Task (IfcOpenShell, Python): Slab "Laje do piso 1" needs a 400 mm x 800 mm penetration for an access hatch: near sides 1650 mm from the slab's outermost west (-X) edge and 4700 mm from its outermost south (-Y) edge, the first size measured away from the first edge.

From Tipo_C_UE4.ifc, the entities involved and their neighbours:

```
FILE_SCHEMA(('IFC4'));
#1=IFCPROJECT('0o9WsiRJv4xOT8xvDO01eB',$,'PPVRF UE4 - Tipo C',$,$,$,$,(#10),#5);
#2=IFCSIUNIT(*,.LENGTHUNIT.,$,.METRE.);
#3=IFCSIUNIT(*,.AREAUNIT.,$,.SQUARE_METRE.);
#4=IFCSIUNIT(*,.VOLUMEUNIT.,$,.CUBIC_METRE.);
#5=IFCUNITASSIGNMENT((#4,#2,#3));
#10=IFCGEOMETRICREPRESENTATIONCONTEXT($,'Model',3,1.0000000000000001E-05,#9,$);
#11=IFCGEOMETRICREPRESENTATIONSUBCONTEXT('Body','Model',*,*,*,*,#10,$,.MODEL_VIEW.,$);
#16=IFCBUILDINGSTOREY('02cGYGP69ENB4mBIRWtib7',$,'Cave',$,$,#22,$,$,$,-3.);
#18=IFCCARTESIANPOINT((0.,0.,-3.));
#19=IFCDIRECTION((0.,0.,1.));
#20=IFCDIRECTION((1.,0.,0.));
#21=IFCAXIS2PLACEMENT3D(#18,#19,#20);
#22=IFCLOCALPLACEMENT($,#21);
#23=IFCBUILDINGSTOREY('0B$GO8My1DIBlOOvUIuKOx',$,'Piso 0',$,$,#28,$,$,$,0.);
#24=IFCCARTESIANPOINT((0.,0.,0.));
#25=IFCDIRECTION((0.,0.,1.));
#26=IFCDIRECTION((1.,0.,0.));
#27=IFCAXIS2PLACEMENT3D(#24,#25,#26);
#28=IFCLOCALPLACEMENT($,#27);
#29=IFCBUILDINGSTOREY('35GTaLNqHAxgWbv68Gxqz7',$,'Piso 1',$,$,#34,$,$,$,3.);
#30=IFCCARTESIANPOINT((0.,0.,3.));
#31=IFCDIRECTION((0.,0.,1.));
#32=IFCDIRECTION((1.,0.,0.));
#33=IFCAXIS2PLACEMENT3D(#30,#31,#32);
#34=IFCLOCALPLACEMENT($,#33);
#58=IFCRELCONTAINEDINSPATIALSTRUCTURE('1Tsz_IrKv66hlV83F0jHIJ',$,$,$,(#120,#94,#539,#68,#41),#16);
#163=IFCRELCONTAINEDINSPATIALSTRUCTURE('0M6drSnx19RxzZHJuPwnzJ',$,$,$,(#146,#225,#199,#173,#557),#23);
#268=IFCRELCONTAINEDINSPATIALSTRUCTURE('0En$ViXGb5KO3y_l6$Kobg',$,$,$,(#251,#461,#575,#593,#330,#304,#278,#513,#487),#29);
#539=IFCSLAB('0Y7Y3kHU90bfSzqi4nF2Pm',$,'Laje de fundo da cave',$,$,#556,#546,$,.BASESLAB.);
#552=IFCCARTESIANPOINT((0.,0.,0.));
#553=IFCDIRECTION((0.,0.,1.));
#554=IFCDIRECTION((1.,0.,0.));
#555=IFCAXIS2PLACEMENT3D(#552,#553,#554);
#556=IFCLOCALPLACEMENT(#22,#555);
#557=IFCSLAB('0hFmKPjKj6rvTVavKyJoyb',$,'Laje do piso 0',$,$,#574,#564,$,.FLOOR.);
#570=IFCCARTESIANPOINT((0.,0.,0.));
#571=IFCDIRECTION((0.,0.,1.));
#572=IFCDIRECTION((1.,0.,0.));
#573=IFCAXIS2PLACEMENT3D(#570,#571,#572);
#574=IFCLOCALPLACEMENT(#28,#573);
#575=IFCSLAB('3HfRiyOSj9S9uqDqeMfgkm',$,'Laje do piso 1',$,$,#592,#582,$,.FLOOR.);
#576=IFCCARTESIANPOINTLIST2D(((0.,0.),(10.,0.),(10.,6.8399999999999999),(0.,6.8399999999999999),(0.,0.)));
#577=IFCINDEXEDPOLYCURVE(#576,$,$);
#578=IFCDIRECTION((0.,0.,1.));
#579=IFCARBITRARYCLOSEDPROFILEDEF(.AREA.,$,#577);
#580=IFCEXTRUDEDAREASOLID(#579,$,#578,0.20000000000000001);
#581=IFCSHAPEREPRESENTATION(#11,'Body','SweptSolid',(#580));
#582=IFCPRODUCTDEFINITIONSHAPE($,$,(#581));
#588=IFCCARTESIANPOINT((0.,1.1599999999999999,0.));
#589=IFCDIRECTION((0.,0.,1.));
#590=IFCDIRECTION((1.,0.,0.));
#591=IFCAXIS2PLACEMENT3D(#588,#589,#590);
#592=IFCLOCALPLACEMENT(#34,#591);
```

```python
import numpy as np
import ifcopenshell
import ifcopenshell.api.feature
import ifcopenshell.api.geometry
import ifcopenshell.api.root
import ifcopenshell.geom
import ifcopenshell.util.placement
import ifcopenshell.util.representation
import ifcopenshell.util.shape
import ifcopenshell.util.unit

model = ifcopenshell.open("Tipo_C_UE4.ifc")
unit_scale = ifcopenshell.util.unit.calculate_unit_scale(model)
settings = ifcopenshell.geom.settings()


def volume(element):
    """Net volume in cubic metres, openings subtracted."""
    shape = ifcopenshell.geom.create_shape(settings, element)
    return ifcopenshell.util.shape.get_volume(shape.geometry)


slab = model.by_guid("3HfRiyOSj9S9uqDqeMfgkm")
before = volume(slab)

# Extent in the slab's own axes, in metres. The edges named are its -X and -Y sides.
slab_shape = ifcopenshell.geom.create_shape(settings, slab)
vertices = ifcopenshell.util.shape.get_vertices(slab_shape.geometry)
x_min, y_min, bottom = vertices.min(axis=0)
top = vertices[:, 2].max()

opening = ifcopenshell.api.root.create_entity(model, ifc_class="IfcOpeningElement", name="Access hatch opening", predefined_type="OPENING")
context = ifcopenshell.util.representation.get_context(model, "Model", "Body", "MODEL_VIEW")
width, depth = 0.4, 0.8
outline = [(0.0, 0.0), (width, 0.0), (width, depth), (0.0, depth), (0.0, 0.0)]
# Overshoot both faces by 50 mm so the cut is clean.
shape = ifcopenshell.api.geometry.add_slab_representation(
    model, context=context, depth=top - bottom + 0.1, polyline=outline
)
ifcopenshell.api.geometry.assign_representation(model, product=opening, representation=shape)

matrix = ifcopenshell.util.placement.get_local_placement(slab.ObjectPlacement)
matrix[:, 3] = matrix @ np.append(np.array([x_min + 1.65, y_min + 4.7, bottom - 0.05]) / unit_scale, 1.0)
ifcopenshell.api.geometry.edit_object_placement(model, product=opening, matrix=matrix, is_si=False)
ifcopenshell.api.feature.add_feature(model, feature=opening, element=slab)

after = volume(slab)

print(f"slab volume {before:.3f} -> {after:.3f} m3")

model.write("Tipo_C_UE4_updated.ifc")
```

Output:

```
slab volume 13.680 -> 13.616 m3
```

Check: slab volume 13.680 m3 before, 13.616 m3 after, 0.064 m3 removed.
